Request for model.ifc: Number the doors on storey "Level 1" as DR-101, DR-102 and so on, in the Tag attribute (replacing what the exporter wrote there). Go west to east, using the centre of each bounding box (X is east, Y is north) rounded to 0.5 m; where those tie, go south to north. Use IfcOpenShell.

First a look at what the model holds.

```python
import ifcopenshell
import ifcopenshell.util.element
import ifcopenshell.util.placement

model = ifcopenshell.open("model.ifc")
print(model.schema)
storey = next(s for s in model.by_type("IfcBuildingStorey") if s.Name == "Level 1")
doors = [e for e in ifcopenshell.util.element.get_decomposition(storey) if e.is_a("IfcDoor")]
for e in sorted(doors, key=lambda e: e.id()):
    origin = ifcopenshell.util.placement.get_local_placement(e.ObjectPlacement)[:3, 3]
    print(e.id(), e.Tag, e.Name, origin.round(2) + 0.0, sep=" | ")
```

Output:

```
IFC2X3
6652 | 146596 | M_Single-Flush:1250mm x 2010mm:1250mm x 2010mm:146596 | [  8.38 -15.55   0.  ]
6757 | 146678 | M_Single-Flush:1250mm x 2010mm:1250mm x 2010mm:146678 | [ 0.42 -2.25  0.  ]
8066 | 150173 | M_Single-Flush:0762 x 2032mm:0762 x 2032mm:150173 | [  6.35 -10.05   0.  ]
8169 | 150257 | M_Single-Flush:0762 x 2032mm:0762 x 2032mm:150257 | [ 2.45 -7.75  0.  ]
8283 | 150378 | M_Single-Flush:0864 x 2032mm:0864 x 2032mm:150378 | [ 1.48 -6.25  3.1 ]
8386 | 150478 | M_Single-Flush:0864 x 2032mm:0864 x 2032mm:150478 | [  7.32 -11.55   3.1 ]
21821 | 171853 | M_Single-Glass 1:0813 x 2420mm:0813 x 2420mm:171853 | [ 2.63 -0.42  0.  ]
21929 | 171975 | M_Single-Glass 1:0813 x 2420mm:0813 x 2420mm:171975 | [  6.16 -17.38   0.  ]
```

```python
import ifcopenshell
import ifcopenshell.geom
import ifcopenshell.util.element
import ifcopenshell.util.shape

model = ifcopenshell.open("model.ifc")
settings = ifcopenshell.geom.settings()
settings.set("use-world-coords", True)


def centre(element):
    shape = ifcopenshell.geom.create_shape(settings, element)
    return ifcopenshell.util.shape.get_bbox_centroid(shape.geometry)


storey = next(s for s in model.by_type("IfcBuildingStorey") if s.Name == "Level 1")
doors = [e for e in ifcopenshell.util.element.get_decomposition(storey) if e.is_a("IfcDoor")]

# Insertion points can sit at a corner or the storey origin, so sort by the geometry (in metres).
centres = {e: centre(e) for e in doors}
doors.sort(key=lambda e: (round(centres[e][0] / 0.5), centres[e][1]))

for i, e in enumerate(doors, start=1):
    number = f"DR-1{i:02d}"
    e.Tag = number
    print(e.id(), number)

model.write("model_edited.ifc")
```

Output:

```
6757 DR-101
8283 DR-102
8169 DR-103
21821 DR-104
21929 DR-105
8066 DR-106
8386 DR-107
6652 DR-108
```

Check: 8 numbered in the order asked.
